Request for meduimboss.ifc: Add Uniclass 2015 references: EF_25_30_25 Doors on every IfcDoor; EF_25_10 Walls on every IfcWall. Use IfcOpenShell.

First a look at what the model holds.

```python
import ifcopenshell

model = ifcopenshell.open("meduimboss.ifc")
print(model.schema)
print("classifications:", [c.Name for c in model.by_type("IfcClassification")])
for ifc_class in ("IfcDoor", "IfcRoof", "IfcStair", "IfcWall", "IfcWindow"):
    print(ifc_class, len(model.by_type(ifc_class)))
```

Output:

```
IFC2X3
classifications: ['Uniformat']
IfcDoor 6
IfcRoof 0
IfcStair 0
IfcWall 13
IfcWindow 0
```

```python
import ifcopenshell
import ifcopenshell.api.classification

model = ifcopenshell.open("meduimboss.ifc")

# IFC2X3 requires Source and Edition and has no link from the project to the system.
system = model.create_entity("IfcClassification", Source="NBS", Edition="2015", Name="Uniclass 2015")

codes = {
    "IfcDoor": ("EF_25_30_25", "Doors"),
    "IfcWall": ("EF_25_10", "Walls"),
}
for ifc_class, (code, name) in codes.items():
    products = model.by_type(ifc_class)
    ifcopenshell.api.classification.add_reference(
        model, products=products, classification=system, identification=code, name=name
    )
    print(code, len(products))

model.write("meduimboss_updated.ifc")
```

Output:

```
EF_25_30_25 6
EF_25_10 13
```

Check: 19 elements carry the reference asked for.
